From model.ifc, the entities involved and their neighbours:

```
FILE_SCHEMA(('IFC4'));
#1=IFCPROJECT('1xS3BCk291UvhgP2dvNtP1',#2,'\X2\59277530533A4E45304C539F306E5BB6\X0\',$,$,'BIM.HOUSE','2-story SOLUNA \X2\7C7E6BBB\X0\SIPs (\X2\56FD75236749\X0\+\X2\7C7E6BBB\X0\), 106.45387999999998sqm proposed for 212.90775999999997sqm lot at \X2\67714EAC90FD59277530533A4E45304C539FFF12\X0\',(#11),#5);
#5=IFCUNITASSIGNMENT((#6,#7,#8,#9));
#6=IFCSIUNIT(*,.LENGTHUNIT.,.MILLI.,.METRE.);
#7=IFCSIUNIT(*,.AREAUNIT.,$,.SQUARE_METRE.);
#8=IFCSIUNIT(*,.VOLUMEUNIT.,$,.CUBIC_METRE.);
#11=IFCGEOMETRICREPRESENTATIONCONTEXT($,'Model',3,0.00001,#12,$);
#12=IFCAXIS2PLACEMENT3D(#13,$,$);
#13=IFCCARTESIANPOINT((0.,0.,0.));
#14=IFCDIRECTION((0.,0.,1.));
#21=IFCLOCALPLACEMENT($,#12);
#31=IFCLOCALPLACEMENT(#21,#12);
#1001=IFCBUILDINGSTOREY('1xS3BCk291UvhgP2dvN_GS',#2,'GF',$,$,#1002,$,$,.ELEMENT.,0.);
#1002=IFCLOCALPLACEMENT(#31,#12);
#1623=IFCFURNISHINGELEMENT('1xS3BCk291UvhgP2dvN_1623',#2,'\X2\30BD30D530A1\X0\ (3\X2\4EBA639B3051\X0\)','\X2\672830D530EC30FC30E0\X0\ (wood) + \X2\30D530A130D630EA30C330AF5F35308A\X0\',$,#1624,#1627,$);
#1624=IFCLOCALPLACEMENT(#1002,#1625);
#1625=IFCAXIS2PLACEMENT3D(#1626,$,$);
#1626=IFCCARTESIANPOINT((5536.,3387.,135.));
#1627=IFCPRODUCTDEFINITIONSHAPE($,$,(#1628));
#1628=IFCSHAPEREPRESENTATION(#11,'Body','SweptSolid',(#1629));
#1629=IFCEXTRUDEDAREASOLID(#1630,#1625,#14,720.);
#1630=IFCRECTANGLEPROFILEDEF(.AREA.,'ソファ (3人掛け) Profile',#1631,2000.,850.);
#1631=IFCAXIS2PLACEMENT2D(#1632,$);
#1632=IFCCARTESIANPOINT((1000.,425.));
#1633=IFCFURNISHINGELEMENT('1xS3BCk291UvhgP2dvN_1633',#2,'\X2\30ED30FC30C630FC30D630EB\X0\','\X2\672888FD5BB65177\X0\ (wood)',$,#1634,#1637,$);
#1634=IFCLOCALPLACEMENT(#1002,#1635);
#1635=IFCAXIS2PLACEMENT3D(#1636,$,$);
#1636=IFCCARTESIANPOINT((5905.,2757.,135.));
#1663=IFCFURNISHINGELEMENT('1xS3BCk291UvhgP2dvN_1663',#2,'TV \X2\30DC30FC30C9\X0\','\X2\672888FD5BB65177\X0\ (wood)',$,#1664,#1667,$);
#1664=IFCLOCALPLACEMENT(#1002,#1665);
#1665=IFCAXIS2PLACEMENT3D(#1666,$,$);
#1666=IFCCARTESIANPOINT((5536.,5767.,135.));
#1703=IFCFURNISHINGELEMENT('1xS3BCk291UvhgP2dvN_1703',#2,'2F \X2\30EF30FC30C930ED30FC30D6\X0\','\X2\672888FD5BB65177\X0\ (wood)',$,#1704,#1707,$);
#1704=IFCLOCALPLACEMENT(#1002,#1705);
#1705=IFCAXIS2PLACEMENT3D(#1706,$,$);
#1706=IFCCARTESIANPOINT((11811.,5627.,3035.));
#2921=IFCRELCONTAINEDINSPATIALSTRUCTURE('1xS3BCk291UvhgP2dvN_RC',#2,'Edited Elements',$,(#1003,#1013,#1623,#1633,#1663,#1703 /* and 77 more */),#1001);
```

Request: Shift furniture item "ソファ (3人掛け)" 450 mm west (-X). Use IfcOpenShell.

```python
import ifcopenshell
import ifcopenshell.api.geometry
import ifcopenshell.util.placement
import ifcopenshell.util.unit

model = ifcopenshell.open("model.ifc")
unit_scale = ifcopenshell.util.unit.calculate_unit_scale(model)

item = model.by_guid("1xS3BCk291UvhgP2dvN_1623")
matrix = ifcopenshell.util.placement.get_local_placement(item.ObjectPlacement)
matrix[0, 3] -= 0.45 / unit_scale
ifcopenshell.api.geometry.edit_object_placement(model, product=item, matrix=matrix, is_si=False)

print(ifcopenshell.util.placement.get_local_placement(item.ObjectPlacement).round(3) + 0.0)

model.write("model_v2.ifc")
```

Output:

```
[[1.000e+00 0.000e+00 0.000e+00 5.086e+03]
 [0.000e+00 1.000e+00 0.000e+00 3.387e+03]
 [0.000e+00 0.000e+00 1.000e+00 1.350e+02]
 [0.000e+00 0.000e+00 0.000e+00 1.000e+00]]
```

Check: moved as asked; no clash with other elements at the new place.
